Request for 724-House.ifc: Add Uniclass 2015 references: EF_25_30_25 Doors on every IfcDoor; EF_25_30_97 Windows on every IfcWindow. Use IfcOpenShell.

First a look at what the model holds.

```python
import ifcopenshell

model = ifcopenshell.open("724-House.ifc")
print(model.schema)
print("classifications:", [c.Name for c in model.by_type("IfcClassification")])
for ifc_class in ("IfcDoor", "IfcRoof", "IfcStair", "IfcWall", "IfcWindow"):
    print(ifc_class, len(model.by_type(ifc_class)))
```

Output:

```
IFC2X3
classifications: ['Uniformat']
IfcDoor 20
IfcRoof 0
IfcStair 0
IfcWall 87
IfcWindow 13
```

```python
import ifcopenshell
import ifcopenshell.api.classification

model = ifcopenshell.open("724-House.ifc")

# IFC2X3 requires Source and Edition and has no link from the project to the system.
system = model.create_entity("IfcClassification", Source="NBS", Edition="2015", Name="Uniclass 2015")

codes = {
    "IfcDoor": ("EF_25_30_25", "Doors"),
    "IfcWindow": ("EF_25_30_97", "Windows"),
}
for ifc_class, (code, name) in codes.items():
    products = model.by_type(ifc_class)
    ifcopenshell.api.classification.add_reference(
        model, products=products, classification=system, identification=code, name=name
    )
    print(code, len(products))

model.write("724-House_edited.ifc")
```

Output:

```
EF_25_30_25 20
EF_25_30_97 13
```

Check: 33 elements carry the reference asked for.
